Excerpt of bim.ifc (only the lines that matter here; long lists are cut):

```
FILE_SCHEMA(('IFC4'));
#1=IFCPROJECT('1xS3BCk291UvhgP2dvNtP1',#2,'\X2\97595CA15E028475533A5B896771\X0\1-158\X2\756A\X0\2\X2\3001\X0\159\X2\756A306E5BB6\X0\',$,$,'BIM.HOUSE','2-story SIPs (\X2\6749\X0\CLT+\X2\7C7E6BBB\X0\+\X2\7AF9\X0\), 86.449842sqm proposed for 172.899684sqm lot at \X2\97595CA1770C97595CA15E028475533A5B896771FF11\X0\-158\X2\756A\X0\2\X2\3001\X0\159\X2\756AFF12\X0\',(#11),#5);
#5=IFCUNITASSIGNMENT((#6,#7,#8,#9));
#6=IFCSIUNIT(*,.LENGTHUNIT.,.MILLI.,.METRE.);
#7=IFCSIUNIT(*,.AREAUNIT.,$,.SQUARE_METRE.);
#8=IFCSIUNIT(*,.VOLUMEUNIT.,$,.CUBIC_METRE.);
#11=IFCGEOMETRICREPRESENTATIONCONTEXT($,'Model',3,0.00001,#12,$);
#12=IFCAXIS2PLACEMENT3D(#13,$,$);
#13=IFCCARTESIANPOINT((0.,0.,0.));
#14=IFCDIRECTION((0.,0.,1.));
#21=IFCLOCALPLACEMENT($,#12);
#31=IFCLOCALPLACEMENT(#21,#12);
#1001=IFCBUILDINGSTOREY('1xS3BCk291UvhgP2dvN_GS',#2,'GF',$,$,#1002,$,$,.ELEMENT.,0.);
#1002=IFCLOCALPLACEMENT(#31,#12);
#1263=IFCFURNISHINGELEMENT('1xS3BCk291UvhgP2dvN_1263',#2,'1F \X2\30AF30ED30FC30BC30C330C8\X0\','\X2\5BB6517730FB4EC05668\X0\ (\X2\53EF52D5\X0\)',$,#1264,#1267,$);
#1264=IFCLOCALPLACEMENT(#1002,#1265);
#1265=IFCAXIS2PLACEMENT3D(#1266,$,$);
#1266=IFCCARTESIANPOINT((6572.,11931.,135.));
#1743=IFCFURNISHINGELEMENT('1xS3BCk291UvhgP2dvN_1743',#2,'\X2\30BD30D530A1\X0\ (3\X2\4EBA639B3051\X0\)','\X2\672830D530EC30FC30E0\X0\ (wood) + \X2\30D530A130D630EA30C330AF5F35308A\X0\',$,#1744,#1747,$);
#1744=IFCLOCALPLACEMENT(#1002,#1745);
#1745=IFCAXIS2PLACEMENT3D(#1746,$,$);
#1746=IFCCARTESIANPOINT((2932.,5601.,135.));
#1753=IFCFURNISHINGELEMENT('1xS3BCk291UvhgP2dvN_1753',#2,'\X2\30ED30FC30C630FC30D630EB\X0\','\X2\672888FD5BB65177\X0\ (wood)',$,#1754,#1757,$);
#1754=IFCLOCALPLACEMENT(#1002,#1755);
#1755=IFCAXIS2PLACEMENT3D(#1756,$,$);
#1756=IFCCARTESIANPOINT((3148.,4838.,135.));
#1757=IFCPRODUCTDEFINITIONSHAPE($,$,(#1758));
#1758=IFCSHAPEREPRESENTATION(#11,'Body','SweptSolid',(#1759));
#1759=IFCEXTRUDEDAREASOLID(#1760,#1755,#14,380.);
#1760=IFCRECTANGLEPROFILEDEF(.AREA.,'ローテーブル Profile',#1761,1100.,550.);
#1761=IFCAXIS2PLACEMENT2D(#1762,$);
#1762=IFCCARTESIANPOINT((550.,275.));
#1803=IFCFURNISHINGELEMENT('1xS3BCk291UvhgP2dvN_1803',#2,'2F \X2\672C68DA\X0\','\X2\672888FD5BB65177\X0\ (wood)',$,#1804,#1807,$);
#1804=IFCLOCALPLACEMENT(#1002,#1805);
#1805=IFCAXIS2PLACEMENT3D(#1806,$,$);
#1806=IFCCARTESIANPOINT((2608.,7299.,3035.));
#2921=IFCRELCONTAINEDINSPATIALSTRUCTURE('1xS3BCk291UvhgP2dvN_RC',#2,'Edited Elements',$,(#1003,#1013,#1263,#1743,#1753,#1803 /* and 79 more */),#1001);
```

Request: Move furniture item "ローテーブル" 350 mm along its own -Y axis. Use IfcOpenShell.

```python
import ifcopenshell
import ifcopenshell.api.geometry
import ifcopenshell.util.placement
import ifcopenshell.util.unit

model = ifcopenshell.open("bim.ifc")
unit_scale = ifcopenshell.util.unit.calculate_unit_scale(model)

item = model.by_guid("1xS3BCk291UvhgP2dvN_1753")
matrix = ifcopenshell.util.placement.get_local_placement(item.ObjectPlacement)
matrix[:3, 3] -= matrix[:3, 1] * 0.35 / unit_scale
ifcopenshell.api.geometry.edit_object_placement(model, product=item, matrix=matrix, is_si=False)

print(ifcopenshell.util.placement.get_local_placement(item.ObjectPlacement).round(3) + 0.0)

model.write("bim_rev.ifc")
```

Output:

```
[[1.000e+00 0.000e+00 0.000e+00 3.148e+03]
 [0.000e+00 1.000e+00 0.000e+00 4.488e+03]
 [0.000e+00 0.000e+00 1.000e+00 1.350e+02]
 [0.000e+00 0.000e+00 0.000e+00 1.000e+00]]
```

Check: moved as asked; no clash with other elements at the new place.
